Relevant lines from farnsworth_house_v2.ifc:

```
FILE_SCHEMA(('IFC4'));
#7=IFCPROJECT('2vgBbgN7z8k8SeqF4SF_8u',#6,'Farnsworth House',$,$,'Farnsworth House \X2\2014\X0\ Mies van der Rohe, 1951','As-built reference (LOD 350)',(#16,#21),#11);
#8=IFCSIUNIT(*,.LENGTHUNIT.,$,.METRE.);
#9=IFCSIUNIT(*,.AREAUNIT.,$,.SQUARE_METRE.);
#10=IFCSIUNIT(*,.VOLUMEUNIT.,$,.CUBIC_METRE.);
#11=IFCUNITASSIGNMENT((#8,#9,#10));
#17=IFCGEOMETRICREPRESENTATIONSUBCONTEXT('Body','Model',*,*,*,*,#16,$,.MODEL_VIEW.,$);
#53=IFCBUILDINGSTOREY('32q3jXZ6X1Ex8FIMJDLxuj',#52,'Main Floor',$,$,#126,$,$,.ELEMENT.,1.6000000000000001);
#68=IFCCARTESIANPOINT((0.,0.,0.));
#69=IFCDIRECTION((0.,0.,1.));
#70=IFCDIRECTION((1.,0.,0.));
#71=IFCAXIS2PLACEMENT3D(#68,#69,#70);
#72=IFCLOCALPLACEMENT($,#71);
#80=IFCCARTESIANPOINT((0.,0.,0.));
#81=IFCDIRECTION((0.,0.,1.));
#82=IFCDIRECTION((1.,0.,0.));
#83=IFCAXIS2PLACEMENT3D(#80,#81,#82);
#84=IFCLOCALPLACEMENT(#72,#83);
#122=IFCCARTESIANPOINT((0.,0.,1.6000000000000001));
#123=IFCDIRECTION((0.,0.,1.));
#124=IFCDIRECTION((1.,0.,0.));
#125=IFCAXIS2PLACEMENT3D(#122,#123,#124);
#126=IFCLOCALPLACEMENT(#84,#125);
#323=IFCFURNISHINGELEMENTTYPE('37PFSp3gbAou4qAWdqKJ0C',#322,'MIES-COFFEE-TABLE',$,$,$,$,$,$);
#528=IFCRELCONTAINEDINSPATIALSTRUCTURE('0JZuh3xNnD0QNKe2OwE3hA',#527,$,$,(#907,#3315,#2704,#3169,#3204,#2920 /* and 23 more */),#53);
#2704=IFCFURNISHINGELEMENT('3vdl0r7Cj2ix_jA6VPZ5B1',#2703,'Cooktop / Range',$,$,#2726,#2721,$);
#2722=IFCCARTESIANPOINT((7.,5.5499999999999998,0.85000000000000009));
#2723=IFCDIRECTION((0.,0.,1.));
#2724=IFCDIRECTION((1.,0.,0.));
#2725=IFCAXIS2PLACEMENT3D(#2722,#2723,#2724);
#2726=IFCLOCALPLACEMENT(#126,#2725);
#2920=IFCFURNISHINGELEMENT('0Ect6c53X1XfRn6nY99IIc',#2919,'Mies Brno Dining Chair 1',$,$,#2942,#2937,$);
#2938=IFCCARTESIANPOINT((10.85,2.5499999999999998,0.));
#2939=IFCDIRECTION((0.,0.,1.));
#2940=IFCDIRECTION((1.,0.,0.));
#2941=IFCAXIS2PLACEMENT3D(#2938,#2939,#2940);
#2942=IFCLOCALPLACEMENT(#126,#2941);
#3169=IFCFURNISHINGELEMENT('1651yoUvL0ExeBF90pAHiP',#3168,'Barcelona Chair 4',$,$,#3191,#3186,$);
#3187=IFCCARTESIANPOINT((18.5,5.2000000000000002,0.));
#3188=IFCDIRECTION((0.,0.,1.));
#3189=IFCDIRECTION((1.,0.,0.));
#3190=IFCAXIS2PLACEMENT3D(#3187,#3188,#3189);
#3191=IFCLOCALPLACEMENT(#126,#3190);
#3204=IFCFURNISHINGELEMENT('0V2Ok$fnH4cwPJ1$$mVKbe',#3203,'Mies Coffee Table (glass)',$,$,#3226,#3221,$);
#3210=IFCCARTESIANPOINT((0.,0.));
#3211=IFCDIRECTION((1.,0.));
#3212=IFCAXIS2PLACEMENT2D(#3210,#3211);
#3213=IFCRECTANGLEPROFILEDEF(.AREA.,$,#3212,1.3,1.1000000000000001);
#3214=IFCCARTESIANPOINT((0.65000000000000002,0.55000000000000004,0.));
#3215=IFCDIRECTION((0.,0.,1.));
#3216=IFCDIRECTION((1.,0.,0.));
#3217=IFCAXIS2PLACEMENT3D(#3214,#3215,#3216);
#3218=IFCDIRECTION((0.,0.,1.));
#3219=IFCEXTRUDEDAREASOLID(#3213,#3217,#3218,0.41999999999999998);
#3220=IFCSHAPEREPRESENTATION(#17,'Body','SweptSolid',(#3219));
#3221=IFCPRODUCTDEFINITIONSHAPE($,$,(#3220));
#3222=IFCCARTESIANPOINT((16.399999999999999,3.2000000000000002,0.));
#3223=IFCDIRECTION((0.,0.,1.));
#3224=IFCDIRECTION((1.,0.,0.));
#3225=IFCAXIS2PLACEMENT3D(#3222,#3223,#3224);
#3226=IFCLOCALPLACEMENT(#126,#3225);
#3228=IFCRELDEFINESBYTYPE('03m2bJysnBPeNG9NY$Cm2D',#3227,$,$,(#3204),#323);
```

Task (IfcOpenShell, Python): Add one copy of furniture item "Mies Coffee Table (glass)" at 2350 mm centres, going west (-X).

```python
import numpy as np
import ifcopenshell
import ifcopenshell.api.geometry
import ifcopenshell.api.root
import ifcopenshell.util.element
import ifcopenshell.util.placement
import ifcopenshell.util.unit

model = ifcopenshell.open("farnsworth_house_v2.ifc")
unit_scale = ifcopenshell.util.unit.calculate_unit_scale(model)


def reuse_history(source, copy):
    """copy_class also copies each property set's owner history, people and application; keep the originals."""
    for rel in copy.IsDefinedBy:
        if rel.is_a("IfcRelDefinesByProperties") and (history := rel.RelatingPropertyDefinition.OwnerHistory):
            rel.RelatingPropertyDefinition.OwnerHistory = source.OwnerHistory
            ifcopenshell.util.element.remove_deep2(model, history)


source = model.by_guid("0V2Ok$fnH4cwPJ1$$mVKbe")
base = ifcopenshell.util.placement.get_local_placement(source.ObjectPlacement)
step = np.array([-1.0, 0.0, 0.0]) * 2.35 / unit_scale

for i in range(1, 2):
    copy = ifcopenshell.api.root.copy_class(model, product=source)
    copy.Representation = ifcopenshell.util.element.copy_deep(
        model, source.Representation, exclude=["IfcGeometricRepresentationContext", "IfcRepresentationMap"]
    )
    reuse_history(source, copy)
    matrix = base.copy()
    matrix[:3, 3] += i * step
    print("added at", matrix[:3, 3].round(3) + 0.0)
    ifcopenshell.api.geometry.edit_object_placement(model, product=copy, matrix=matrix, is_si=False)

model.write("farnsworth_house_v2_rev.ifc")
```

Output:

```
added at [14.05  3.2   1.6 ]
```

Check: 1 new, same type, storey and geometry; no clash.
